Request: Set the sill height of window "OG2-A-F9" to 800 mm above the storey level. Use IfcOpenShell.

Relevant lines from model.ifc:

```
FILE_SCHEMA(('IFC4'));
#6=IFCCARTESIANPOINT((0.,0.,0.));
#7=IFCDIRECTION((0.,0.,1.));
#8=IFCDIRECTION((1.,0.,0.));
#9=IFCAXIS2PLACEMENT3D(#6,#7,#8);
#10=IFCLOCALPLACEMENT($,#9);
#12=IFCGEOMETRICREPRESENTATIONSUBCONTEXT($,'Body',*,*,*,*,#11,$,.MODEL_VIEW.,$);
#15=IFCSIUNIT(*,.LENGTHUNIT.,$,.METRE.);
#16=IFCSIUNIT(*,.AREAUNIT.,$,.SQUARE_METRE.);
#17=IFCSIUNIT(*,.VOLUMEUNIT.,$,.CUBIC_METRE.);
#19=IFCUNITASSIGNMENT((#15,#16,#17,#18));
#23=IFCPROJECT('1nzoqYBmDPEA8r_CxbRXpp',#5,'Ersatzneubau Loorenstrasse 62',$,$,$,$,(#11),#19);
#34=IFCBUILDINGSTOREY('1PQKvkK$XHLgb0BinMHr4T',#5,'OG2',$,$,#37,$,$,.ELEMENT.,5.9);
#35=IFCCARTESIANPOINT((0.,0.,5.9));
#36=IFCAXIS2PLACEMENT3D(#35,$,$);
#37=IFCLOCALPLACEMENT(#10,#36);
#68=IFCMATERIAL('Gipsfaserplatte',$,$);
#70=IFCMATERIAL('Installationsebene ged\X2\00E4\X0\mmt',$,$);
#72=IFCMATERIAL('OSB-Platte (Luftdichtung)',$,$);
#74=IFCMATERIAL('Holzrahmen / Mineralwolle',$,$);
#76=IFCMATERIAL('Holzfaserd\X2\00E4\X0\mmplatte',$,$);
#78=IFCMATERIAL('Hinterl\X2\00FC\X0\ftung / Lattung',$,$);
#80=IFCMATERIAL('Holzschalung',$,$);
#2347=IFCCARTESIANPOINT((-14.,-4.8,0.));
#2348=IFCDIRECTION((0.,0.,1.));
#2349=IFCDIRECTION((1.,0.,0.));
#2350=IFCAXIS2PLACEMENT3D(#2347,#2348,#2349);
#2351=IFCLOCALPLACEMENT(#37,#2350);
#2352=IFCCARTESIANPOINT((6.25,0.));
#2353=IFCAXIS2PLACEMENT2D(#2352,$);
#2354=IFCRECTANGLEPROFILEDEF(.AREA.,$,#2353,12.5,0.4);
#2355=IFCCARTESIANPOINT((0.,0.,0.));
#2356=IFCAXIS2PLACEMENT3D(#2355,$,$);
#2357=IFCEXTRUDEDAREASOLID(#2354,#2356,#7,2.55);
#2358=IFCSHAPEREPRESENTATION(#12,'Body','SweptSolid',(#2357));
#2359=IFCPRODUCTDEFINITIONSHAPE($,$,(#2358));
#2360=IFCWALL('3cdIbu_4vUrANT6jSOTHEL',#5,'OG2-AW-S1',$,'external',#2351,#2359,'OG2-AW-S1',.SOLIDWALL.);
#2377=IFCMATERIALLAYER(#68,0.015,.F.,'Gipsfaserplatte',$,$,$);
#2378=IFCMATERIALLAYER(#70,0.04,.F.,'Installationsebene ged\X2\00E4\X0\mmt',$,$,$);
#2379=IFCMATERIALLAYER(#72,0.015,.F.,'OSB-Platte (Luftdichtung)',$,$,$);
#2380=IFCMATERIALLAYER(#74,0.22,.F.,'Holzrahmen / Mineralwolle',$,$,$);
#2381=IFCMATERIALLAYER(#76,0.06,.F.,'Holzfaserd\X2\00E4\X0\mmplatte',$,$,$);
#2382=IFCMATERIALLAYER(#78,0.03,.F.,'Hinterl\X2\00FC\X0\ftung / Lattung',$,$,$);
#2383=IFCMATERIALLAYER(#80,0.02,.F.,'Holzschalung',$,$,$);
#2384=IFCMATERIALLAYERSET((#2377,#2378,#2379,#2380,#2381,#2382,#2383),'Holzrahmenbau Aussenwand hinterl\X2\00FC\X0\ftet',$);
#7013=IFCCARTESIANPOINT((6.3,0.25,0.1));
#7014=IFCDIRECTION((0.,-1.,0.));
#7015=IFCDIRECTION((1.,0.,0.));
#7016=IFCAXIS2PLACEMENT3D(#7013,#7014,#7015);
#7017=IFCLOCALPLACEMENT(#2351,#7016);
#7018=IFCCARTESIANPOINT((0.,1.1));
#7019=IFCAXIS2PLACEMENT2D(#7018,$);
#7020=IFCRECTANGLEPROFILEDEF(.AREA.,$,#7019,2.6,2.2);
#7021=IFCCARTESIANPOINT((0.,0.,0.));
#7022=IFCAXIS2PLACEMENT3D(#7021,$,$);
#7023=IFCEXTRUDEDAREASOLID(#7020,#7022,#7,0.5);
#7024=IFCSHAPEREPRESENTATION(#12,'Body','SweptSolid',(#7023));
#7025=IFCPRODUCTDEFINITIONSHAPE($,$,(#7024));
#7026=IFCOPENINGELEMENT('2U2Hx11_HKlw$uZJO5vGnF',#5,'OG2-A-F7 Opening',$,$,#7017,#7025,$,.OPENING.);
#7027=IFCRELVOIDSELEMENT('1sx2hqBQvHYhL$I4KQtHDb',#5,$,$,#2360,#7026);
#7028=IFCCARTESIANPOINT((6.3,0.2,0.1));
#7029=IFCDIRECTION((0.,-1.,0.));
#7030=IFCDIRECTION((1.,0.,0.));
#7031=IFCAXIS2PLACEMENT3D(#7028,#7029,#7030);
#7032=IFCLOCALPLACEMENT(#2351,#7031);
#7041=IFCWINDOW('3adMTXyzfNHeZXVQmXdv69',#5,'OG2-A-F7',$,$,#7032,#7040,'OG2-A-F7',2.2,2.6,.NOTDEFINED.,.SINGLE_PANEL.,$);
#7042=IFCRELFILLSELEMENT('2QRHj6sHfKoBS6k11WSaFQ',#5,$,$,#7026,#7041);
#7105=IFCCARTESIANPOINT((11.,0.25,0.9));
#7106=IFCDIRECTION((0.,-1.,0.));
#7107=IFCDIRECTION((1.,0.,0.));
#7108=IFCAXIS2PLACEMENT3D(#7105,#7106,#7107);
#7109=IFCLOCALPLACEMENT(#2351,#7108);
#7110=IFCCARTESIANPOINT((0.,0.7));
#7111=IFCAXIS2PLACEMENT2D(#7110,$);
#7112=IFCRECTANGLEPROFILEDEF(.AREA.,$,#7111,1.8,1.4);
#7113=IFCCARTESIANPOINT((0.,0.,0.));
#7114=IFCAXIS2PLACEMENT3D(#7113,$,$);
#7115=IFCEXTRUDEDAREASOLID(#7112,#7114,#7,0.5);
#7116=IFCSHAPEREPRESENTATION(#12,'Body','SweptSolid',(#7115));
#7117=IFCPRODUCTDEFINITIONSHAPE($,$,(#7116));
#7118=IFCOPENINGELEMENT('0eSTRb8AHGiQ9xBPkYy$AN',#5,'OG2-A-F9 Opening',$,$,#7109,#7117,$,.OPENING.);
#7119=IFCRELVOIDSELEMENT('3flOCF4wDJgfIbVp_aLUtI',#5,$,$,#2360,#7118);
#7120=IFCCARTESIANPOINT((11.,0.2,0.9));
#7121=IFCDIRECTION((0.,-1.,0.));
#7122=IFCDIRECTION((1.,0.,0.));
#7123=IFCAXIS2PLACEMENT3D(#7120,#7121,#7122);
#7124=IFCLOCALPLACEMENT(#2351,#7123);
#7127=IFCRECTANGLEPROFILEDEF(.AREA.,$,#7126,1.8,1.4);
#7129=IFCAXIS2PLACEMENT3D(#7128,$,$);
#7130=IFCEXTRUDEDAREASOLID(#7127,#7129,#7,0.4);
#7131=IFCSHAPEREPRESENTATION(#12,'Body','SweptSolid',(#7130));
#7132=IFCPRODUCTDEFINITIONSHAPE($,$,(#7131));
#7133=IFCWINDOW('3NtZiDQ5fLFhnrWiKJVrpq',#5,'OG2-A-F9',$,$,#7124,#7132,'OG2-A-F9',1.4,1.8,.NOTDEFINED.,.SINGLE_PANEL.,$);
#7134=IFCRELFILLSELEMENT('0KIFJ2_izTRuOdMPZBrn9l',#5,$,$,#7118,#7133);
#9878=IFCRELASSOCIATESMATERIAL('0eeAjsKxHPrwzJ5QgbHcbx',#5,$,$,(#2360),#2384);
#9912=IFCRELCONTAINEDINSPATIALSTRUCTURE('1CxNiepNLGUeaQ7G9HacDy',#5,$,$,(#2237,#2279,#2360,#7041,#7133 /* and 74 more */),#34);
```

```python
import numpy as np
import ifcopenshell
import ifcopenshell.api.geometry
import ifcopenshell.geom
import ifcopenshell.util.element
import ifcopenshell.util.placement
import ifcopenshell.util.shape
import ifcopenshell.util.unit

model = ifcopenshell.open("model.ifc")
unit_scale = ifcopenshell.util.unit.calculate_unit_scale(model)

window = model.by_guid("3NtZiDQ5fLFhnrWiKJVrpq")
opening = window.FillsVoids[0].RelatingOpeningElement
storey = ifcopenshell.util.element.get_container(window, ifc_class="IfcBuildingStorey")
level = ifcopenshell.util.placement.get_local_placement(storey.ObjectPlacement)[2, 3]

# The opening's origin need not be at the sill, so measure its lowest point.
shape = ifcopenshell.geom.create_shape(ifcopenshell.geom.settings(), opening)
bottom = ifcopenshell.util.shape.get_shape_bottom_elevation(shape, shape.geometry) / unit_scale
dz = level + 0.8 / unit_scale - bottom

shift = np.array([0.0, 0.0, dz])
# The window is not placed relative to its opening, so move both.
for product in (opening, window):
    matrix = ifcopenshell.util.placement.get_local_placement(product.ObjectPlacement)
    matrix[:3, 3] += shift
    ifcopenshell.api.geometry.edit_object_placement(model, product=product, matrix=matrix, is_si=False)

print(f"moved by {dz * unit_scale:+.3f} m")

model.write("model_edited.ifc")
```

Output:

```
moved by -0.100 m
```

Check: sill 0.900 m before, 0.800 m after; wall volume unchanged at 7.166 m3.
